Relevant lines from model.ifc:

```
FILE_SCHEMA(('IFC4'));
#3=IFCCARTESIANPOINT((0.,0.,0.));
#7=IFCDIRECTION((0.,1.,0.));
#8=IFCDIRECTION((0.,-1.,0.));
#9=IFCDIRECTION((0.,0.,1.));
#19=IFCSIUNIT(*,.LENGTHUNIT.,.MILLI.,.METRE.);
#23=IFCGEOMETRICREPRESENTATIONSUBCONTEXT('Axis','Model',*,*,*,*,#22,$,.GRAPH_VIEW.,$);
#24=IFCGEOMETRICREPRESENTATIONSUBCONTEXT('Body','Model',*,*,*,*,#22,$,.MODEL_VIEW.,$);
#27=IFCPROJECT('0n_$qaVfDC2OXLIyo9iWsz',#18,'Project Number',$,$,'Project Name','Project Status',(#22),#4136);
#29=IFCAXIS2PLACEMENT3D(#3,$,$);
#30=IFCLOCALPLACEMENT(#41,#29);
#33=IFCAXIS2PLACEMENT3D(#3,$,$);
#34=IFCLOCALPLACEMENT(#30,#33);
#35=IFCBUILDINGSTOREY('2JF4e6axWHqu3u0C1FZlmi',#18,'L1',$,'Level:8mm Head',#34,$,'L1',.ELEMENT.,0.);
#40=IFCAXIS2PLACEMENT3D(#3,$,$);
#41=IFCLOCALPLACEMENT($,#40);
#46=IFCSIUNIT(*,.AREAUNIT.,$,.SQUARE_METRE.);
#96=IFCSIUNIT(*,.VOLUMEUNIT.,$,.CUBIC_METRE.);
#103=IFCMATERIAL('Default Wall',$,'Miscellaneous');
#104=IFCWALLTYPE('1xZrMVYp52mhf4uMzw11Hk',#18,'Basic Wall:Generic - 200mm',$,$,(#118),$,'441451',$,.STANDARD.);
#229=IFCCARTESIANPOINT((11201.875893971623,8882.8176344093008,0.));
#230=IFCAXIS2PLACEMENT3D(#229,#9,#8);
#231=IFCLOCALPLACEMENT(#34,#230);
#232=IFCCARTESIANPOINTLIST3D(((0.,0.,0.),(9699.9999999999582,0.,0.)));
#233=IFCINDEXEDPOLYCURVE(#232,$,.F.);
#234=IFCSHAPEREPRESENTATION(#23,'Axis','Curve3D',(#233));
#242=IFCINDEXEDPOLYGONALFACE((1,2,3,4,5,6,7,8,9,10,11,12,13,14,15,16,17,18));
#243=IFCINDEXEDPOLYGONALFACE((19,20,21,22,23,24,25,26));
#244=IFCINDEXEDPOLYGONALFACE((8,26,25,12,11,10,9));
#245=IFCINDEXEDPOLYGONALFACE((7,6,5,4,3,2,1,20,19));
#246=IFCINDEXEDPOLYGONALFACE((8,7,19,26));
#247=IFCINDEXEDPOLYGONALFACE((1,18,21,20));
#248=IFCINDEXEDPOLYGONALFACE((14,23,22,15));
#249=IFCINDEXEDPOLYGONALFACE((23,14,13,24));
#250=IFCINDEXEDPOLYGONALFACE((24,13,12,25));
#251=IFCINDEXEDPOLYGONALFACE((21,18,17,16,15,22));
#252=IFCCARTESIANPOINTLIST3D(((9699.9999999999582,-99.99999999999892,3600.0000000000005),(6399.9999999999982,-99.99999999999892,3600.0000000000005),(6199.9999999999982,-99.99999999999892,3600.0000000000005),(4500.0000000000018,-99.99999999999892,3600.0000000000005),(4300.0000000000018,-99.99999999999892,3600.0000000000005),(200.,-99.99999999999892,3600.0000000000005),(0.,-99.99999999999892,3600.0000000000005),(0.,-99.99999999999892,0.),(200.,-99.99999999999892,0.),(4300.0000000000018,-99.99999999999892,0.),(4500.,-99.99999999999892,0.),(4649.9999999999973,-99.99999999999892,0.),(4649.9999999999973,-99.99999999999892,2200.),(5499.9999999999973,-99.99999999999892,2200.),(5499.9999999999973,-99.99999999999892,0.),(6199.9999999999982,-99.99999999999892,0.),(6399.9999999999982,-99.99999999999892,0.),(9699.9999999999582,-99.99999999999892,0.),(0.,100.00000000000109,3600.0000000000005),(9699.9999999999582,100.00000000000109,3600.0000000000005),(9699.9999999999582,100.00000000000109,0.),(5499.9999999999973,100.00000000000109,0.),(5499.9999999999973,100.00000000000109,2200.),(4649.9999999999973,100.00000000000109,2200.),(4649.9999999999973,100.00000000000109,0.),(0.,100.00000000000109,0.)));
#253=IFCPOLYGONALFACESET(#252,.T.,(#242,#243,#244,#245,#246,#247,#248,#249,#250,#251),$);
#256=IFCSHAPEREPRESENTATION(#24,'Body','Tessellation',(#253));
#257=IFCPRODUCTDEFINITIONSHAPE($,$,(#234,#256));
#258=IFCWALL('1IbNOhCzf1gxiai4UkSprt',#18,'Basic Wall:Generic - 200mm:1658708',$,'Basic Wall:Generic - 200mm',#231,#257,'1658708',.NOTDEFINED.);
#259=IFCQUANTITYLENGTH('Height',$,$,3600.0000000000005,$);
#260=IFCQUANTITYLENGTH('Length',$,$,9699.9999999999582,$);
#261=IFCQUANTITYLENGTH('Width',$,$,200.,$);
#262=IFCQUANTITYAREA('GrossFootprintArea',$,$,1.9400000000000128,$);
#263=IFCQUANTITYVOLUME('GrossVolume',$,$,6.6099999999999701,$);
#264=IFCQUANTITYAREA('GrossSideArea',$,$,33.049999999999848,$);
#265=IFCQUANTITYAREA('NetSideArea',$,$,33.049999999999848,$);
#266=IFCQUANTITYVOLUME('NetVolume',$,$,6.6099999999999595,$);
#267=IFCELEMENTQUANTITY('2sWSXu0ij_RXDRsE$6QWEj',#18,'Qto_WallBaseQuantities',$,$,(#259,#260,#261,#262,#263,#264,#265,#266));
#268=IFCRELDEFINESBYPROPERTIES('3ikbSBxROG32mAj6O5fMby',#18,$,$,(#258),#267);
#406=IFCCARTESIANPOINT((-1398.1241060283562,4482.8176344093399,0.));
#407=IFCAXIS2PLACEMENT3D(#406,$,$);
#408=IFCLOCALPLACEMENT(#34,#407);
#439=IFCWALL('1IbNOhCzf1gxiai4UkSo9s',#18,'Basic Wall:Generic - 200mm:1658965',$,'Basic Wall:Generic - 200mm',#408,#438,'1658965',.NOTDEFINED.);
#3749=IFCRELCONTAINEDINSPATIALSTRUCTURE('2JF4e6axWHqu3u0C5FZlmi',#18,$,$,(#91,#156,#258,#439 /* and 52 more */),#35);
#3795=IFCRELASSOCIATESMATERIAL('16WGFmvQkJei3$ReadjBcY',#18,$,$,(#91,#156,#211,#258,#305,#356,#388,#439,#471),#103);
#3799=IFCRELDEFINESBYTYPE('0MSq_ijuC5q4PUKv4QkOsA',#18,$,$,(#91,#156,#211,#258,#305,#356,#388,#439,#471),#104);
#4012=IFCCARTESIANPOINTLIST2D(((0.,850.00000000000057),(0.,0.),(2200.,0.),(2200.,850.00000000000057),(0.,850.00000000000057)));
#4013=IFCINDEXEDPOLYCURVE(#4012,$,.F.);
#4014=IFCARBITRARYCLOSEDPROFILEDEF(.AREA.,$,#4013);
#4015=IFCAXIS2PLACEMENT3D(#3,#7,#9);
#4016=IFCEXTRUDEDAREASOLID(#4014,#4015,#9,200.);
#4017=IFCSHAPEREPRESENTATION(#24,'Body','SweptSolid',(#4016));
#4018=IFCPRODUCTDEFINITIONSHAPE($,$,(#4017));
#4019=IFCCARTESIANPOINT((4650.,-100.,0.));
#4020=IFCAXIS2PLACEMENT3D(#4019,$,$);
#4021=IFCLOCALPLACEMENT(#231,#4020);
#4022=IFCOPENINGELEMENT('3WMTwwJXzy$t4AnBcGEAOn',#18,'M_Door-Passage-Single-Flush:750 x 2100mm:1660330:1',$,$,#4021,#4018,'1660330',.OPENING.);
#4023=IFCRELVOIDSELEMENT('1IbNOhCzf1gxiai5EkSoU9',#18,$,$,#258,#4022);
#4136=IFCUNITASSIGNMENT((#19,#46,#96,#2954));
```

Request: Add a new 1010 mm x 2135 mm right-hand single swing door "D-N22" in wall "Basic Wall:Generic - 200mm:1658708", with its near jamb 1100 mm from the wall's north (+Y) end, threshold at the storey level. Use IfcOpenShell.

```python
import numpy as np
import ifcopenshell
import ifcopenshell.api.feature
import ifcopenshell.api.geometry
import ifcopenshell.api.pset
import ifcopenshell.api.root
import ifcopenshell.api.spatial
import ifcopenshell.geom
import ifcopenshell.util.element
import ifcopenshell.util.placement
import ifcopenshell.util.representation
import ifcopenshell.util.shape
import ifcopenshell.util.unit

model = ifcopenshell.open("model.ifc")
unit_scale = ifcopenshell.util.unit.calculate_unit_scale(model)
area_scale = ifcopenshell.util.unit.calculate_unit_scale(model, "AREAUNIT")
volume_scale = ifcopenshell.util.unit.calculate_unit_scale(model, "VOLUMEUNIT")
settings = ifcopenshell.geom.settings()


def volume(element):
    """Net volume in cubic metres, openings subtracted."""
    shape = ifcopenshell.geom.create_shape(settings, element)
    return ifcopenshell.util.shape.get_volume(shape.geometry)


wall = model.by_id(258)
storey = ifcopenshell.util.element.get_container(wall, ifc_class="IfcBuildingStorey")
context = ifcopenshell.util.representation.get_context(model, "Model", "Body", "MODEL_VIEW")
before = volume(wall)

width, height, from_end, sill = 1.01, 2.135, 1.1, 0.0  # metres

# The wall runs along its own X axis, and the end named is its -X end.
wall_shape = ifcopenshell.geom.create_shape(settings, wall)
x, y, z = ifcopenshell.util.shape.get_vertices(wall_shape.geometry).T
start = x.min() + from_end
face, thickness = float(y.min()), float(y.max() - y.min())
wall_matrix = ifcopenshell.util.placement.get_local_placement(wall.ObjectPlacement)
level = ifcopenshell.util.placement.get_local_placement(storey.ObjectPlacement)[2, 3]


def in_wall(x, y):
    """Placement at x, y metres in the wall's axes, at sill height."""
    matrix = wall_matrix.copy()
    matrix[:, 3] = wall_matrix @ np.array([x / unit_scale, y / unit_scale, 0.0, 1.0])
    matrix[2, 3] = level + sill / unit_scale
    return matrix


# Opening: a box that overshoots both wall faces by 50 mm.
opening = ifcopenshell.api.root.create_entity(model, ifc_class="IfcOpeningElement", predefined_type="OPENING")
box = ifcopenshell.api.geometry.add_wall_representation(
    model, context=context, length=width, height=height, thickness=thickness + 0.1
)
ifcopenshell.api.geometry.assign_representation(model, product=opening, representation=box)
ifcopenshell.api.geometry.edit_object_placement(model, product=opening, matrix=in_wall(start, face - 0.05), is_si=False)
ifcopenshell.api.feature.add_feature(model, feature=opening, element=wall)

door = ifcopenshell.api.root.create_entity(model, ifc_class="IfcDoor", name="D-N22", predefined_type="DOOR")
door.OverallWidth, door.OverallHeight = width / unit_scale, height / unit_scale
door.OperationType = "SINGLE_SWING_RIGHT"
body = ifcopenshell.api.geometry.add_door_representation(
    model,
    context=context,
    overall_width=door.OverallWidth,
    overall_height=door.OverallHeight,
    operation_type="SINGLE_SWING_RIGHT",
    lining_properties={"LiningDepth": thickness / unit_scale, "ThresholdDepth": thickness / unit_scale},
)
ifcopenshell.api.geometry.assign_representation(model, product=door, representation=body)
ifcopenshell.api.spatial.assign_container(model, products=[door], relating_structure=storey)
ifcopenshell.api.feature.add_filling(model, opening=opening, element=door)

# The lining spans the wall, so the door starts at the wall face.
ifcopenshell.api.geometry.edit_object_placement(model, product=door, matrix=in_wall(start, face), is_si=False)

after = volume(wall)

# Update the wall's stored quantities.
qto = model.by_id(ifcopenshell.util.element.get_pset(wall, "Qto_WallBaseQuantities", should_inherit=False)["id"])
ifcopenshell.api.pset.edit_qto(model, qto=qto, properties={
    "NetSideArea": after / thickness / area_scale,
    "NetVolume": after / volume_scale,
})

print(f"wall volume {before:.3f} -> {after:.3f} m3")

model.write("model_edited.ifc")
```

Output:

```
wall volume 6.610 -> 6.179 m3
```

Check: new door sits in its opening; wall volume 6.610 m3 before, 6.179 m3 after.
